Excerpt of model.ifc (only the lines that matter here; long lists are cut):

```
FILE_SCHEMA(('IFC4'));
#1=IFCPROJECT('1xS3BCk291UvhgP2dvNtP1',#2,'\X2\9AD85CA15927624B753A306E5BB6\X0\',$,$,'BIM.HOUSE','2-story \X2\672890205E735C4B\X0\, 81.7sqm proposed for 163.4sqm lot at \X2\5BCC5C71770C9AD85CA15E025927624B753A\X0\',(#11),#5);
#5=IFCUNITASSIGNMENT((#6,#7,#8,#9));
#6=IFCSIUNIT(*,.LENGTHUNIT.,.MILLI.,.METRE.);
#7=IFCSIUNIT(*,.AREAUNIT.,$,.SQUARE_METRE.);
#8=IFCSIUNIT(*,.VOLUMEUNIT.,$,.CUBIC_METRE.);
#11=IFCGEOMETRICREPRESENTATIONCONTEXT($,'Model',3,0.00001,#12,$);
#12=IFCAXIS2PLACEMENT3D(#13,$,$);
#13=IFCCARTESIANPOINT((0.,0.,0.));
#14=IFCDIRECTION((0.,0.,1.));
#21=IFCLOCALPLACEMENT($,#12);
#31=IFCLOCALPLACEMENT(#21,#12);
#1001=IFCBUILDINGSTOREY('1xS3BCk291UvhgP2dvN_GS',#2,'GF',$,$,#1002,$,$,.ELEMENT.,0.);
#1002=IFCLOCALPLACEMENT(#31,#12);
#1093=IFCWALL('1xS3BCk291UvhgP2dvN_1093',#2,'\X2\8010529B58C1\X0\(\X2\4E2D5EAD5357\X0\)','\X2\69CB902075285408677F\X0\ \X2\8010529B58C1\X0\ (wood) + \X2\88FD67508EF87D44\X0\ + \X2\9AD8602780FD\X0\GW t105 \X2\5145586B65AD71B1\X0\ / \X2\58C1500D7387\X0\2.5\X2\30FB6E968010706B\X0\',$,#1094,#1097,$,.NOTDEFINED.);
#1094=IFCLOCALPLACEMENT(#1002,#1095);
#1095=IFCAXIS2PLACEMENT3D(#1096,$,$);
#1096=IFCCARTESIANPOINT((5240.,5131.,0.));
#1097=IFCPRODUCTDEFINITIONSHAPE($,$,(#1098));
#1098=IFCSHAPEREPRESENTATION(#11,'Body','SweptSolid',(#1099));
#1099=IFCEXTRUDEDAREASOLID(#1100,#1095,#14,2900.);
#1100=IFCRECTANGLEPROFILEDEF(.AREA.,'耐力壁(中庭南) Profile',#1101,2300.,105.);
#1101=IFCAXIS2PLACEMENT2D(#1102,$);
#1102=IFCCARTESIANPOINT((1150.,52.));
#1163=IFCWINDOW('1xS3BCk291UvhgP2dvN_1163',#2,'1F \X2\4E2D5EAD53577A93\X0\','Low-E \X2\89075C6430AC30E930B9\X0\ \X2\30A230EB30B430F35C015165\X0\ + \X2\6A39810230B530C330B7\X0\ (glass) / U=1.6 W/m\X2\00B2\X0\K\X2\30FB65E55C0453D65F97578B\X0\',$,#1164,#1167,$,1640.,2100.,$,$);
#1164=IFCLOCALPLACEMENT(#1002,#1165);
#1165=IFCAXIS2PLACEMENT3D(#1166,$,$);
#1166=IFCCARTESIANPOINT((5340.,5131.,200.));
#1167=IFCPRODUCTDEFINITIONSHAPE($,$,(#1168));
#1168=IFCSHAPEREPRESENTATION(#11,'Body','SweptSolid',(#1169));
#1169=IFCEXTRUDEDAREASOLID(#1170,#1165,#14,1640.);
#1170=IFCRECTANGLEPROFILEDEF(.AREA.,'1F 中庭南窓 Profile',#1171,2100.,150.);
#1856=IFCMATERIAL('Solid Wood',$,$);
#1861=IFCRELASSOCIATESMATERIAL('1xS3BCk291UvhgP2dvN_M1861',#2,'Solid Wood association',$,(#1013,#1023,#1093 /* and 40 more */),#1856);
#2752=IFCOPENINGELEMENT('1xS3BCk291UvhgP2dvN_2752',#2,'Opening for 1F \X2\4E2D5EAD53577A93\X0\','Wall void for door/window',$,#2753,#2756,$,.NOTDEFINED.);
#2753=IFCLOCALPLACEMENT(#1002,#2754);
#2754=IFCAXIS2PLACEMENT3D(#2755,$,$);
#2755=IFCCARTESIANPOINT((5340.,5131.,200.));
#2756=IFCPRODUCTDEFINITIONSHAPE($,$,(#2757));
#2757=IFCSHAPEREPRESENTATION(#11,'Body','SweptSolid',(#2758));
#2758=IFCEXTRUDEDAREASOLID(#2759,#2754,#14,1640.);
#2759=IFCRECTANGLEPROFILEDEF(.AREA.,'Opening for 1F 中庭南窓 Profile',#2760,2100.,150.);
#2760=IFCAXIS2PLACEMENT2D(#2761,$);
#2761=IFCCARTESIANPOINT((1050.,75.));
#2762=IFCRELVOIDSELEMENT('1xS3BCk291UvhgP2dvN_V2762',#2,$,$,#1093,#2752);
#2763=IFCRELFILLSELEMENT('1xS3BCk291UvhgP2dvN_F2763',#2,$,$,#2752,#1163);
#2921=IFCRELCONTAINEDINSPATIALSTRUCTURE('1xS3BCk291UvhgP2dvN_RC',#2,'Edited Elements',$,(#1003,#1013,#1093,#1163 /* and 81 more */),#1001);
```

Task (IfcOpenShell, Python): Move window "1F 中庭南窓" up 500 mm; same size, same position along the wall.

```python
import numpy as np
import ifcopenshell
import ifcopenshell.api.geometry
import ifcopenshell.util.placement
import ifcopenshell.util.unit

model = ifcopenshell.open("model.ifc")
unit_scale = ifcopenshell.util.unit.calculate_unit_scale(model)

window = model.by_id(1163)
opening = window.FillsVoids[0].RelatingOpeningElement
dz = 500.0

shift = np.array([0.0, 0.0, dz])
# The window is not placed relative to its opening, so move both.
for product in (opening, window):
    matrix = ifcopenshell.util.placement.get_local_placement(product.ObjectPlacement)
    matrix[:3, 3] += shift
    ifcopenshell.api.geometry.edit_object_placement(model, product=product, matrix=matrix, is_si=False)

print(f"moved by {dz * unit_scale:+.3f} m")

model.write("model_rev.ifc")
```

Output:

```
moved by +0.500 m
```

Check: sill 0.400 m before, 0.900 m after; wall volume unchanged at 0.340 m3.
